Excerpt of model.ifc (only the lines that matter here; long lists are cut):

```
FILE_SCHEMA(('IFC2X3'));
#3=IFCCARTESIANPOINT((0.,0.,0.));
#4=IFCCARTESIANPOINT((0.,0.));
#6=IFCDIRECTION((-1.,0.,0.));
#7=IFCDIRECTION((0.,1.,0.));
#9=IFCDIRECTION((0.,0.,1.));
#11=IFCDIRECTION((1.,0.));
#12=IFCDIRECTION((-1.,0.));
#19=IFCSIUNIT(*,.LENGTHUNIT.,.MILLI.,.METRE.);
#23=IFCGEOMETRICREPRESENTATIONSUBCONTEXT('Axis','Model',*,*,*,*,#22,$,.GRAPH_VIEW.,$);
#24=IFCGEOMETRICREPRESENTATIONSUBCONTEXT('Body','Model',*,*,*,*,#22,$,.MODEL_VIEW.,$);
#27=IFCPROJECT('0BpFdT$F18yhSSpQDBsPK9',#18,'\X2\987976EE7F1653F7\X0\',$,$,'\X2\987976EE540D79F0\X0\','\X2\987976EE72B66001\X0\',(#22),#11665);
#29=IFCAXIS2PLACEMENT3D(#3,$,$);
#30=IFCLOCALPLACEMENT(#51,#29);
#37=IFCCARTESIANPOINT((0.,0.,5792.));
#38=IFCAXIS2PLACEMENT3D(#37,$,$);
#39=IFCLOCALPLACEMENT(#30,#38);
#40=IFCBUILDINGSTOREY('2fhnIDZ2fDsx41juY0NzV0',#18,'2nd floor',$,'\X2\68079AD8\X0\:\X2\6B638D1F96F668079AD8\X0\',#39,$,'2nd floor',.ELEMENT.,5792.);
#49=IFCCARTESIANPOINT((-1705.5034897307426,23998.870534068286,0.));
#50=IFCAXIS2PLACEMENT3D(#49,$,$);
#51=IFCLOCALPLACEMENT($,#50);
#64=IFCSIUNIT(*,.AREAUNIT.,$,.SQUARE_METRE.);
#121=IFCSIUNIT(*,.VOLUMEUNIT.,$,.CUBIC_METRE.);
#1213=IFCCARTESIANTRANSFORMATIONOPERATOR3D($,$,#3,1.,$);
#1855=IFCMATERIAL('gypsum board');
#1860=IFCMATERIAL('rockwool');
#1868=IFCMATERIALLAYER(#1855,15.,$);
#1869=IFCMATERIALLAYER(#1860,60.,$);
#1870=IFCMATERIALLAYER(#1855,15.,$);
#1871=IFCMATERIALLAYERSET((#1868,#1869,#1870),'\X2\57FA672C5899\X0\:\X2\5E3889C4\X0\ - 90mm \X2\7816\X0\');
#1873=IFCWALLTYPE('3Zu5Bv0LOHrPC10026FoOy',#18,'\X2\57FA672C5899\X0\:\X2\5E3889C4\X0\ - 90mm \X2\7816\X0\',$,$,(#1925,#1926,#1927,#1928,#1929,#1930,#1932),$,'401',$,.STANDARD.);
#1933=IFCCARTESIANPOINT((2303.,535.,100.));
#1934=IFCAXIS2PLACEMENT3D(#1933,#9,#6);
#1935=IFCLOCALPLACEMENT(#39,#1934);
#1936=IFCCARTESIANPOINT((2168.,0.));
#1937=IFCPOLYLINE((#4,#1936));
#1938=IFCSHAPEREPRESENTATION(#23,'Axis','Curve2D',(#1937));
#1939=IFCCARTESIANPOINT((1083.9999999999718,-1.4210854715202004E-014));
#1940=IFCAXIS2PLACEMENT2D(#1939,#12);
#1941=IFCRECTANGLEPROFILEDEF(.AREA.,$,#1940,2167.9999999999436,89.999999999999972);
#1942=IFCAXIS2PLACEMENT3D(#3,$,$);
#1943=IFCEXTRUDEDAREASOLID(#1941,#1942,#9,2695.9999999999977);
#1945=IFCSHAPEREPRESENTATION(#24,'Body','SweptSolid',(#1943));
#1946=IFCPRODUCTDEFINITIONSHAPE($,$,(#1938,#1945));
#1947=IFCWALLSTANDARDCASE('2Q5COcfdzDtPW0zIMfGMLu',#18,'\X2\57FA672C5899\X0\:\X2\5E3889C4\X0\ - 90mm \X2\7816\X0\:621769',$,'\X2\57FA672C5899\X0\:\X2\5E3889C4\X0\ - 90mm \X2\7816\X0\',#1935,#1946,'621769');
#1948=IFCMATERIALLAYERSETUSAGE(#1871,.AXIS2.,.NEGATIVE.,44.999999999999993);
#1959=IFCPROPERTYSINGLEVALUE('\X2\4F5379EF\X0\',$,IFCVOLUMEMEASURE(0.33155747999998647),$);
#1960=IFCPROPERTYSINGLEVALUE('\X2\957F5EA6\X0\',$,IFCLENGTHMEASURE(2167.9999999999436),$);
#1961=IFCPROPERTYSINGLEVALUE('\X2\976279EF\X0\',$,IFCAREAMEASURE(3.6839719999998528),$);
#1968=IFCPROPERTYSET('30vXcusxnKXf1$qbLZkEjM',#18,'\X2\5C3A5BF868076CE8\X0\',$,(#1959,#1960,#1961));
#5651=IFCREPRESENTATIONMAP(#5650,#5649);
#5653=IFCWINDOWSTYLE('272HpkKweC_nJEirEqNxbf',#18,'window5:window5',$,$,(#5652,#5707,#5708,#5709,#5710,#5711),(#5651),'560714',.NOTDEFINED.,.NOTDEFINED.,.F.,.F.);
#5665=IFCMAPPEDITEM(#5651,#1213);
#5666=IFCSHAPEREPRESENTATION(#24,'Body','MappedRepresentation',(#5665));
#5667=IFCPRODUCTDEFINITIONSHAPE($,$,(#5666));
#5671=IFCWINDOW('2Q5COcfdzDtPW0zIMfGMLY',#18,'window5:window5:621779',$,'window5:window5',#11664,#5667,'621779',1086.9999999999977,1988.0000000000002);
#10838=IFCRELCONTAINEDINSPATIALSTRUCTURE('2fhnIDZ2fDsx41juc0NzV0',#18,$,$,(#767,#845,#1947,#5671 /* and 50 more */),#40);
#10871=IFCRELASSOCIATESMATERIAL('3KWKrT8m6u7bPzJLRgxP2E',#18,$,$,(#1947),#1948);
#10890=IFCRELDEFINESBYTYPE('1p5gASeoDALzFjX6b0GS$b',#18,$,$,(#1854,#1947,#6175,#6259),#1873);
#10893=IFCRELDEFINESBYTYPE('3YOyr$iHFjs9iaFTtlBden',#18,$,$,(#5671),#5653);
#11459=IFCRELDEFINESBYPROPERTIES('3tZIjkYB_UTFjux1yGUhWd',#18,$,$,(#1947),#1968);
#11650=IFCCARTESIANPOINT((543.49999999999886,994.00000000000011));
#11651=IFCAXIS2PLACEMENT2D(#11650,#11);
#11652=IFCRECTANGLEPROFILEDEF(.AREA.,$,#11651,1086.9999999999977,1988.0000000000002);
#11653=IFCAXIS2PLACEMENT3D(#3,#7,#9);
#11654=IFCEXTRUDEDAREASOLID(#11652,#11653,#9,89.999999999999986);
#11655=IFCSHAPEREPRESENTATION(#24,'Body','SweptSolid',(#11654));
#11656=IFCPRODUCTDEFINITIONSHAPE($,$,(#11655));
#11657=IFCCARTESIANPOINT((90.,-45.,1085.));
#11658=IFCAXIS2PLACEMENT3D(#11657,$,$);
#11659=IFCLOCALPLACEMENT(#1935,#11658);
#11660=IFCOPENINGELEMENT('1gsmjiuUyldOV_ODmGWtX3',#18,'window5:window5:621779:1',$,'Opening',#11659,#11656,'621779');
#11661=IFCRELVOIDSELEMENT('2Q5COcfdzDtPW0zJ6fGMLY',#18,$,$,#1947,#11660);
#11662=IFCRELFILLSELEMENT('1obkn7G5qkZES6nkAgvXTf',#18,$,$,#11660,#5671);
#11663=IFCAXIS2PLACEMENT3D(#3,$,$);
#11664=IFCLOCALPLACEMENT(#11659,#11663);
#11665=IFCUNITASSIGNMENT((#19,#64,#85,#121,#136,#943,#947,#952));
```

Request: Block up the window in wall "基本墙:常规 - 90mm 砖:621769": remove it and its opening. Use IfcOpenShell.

```python
import ifcopenshell
import ifcopenshell.api.feature
import ifcopenshell.api.pset
import ifcopenshell.api.root
import ifcopenshell.geom
import ifcopenshell.util.element
import ifcopenshell.util.shape
import ifcopenshell.util.unit

model = ifcopenshell.open("model.ifc")
area_scale = ifcopenshell.util.unit.calculate_unit_scale(model, "AREAUNIT")
volume_scale = ifcopenshell.util.unit.calculate_unit_scale(model, "VOLUMEUNIT")
settings = ifcopenshell.geom.settings()


def volume(element):
    """Net volume in cubic metres, openings subtracted."""
    shape = ifcopenshell.geom.create_shape(settings, element)
    return ifcopenshell.util.shape.get_volume(shape.geometry)


window = model.by_id(5671)
opening = window.FillsVoids[0].RelatingOpeningElement
wall = opening.VoidsElements[0].RelatingBuildingElement
before = volume(wall)

ifcopenshell.api.root.remove_product(model, product=window)
ifcopenshell.api.feature.remove_feature(model, feature=opening)

after = volume(wall)
thickness = 0.09  # wall thickness in metres

# Update the wall's stored quantities.
pset = model.by_id(ifcopenshell.util.element.get_pset(wall, "尺寸标注", should_inherit=False)["id"])
ifcopenshell.api.pset.edit_pset(model, pset=pset, properties={
    "体积": model.create_entity("IfcVolumeMeasure", after / volume_scale),
    "面积": model.create_entity("IfcAreaMeasure", after / thickness / area_scale),
})

print(f"wall volume {before:.3f} -> {after:.3f} m3")

model.write("model_v2.ifc")
```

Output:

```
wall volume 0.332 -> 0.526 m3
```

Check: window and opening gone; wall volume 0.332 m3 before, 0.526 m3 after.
